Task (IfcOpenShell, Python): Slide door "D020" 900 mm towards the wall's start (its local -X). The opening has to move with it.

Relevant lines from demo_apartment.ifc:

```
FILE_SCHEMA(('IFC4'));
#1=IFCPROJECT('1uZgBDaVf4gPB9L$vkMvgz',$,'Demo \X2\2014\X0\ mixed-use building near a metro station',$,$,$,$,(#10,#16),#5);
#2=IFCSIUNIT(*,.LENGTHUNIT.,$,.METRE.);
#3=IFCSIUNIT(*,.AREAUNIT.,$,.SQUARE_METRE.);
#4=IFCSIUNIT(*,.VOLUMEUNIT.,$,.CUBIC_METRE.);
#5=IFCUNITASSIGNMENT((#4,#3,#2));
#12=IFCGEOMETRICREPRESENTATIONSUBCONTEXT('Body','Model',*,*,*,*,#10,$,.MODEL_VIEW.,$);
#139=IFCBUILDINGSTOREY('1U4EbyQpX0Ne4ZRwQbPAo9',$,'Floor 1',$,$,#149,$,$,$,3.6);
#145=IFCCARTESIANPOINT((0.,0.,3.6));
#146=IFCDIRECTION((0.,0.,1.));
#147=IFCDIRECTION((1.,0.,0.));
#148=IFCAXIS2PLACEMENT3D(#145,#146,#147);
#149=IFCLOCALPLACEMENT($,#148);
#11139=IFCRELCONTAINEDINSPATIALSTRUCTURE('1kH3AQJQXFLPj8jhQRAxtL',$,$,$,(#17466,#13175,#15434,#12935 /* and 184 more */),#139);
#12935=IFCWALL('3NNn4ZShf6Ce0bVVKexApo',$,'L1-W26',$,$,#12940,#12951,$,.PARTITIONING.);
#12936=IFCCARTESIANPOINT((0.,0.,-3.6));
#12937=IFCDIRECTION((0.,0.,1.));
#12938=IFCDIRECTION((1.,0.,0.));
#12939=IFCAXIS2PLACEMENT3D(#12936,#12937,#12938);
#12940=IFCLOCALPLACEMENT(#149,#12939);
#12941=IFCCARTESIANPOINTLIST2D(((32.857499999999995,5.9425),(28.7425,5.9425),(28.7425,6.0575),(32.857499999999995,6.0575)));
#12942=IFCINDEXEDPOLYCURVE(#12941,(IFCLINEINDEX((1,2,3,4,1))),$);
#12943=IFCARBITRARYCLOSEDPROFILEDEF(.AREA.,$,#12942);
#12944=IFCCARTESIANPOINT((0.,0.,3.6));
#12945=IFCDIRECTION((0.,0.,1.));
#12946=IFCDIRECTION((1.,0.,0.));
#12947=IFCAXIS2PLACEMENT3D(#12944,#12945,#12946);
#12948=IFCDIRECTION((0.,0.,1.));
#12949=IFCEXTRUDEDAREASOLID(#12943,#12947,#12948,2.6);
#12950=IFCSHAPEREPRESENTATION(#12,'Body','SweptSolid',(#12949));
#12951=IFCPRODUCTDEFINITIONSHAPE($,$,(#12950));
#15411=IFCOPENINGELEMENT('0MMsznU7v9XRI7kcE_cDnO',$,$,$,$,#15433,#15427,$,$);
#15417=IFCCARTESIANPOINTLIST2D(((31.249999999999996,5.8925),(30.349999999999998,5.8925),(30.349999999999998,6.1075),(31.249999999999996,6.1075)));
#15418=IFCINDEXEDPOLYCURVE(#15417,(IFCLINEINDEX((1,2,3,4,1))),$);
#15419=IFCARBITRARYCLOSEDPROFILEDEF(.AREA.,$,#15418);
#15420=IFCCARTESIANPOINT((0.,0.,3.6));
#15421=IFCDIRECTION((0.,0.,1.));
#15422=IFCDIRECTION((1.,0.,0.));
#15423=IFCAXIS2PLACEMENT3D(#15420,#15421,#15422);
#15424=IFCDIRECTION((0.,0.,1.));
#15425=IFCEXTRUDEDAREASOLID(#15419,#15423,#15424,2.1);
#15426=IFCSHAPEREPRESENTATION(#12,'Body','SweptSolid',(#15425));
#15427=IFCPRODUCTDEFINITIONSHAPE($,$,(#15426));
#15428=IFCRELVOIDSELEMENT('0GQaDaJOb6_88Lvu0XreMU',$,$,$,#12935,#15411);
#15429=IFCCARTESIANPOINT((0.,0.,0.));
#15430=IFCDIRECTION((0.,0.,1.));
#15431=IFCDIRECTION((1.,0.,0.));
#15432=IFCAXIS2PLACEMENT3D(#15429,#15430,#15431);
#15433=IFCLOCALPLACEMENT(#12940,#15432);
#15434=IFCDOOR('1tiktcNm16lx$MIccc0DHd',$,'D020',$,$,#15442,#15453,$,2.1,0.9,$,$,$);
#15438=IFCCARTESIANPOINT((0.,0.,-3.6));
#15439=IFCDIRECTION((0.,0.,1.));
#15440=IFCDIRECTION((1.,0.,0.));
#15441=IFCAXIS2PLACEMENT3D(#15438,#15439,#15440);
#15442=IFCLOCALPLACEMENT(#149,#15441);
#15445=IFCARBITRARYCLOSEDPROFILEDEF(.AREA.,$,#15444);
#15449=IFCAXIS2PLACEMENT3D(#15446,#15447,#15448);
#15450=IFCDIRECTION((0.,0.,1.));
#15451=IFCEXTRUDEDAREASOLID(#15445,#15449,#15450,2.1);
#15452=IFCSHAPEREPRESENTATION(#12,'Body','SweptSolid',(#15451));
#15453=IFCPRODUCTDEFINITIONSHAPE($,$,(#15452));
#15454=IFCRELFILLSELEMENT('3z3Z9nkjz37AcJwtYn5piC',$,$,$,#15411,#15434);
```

```python
import ifcopenshell
import ifcopenshell.api.geometry
import ifcopenshell.util.placement

model = ifcopenshell.open("demo_apartment.ifc")

door = model.by_guid("1tiktcNm16lx$MIccc0DHd")
opening = door.FillsVoids[0].RelatingOpeningElement
wall = opening.VoidsElements[0].RelatingBuildingElement

wall_matrix = ifcopenshell.util.placement.get_local_placement(wall.ObjectPlacement)
shift = wall_matrix[:3, 0] * -0.9
before = ifcopenshell.util.placement.get_local_placement(door.ObjectPlacement)[:3, 3].copy()

# The door is not placed relative to its opening, so move both.
for product in (opening, door):
    matrix = ifcopenshell.util.placement.get_local_placement(product.ObjectPlacement)
    matrix[:3, 3] += shift
    ifcopenshell.api.geometry.edit_object_placement(model, product=product, matrix=matrix, is_si=False)

after = ifcopenshell.util.placement.get_local_placement(door.ObjectPlacement)[:3, 3]
print("door moved by", (after - before).round(3) + 0.0)

model.write("demo_apartment_updated.ifc")
```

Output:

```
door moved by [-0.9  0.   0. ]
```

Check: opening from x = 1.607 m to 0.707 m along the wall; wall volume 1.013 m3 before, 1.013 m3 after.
